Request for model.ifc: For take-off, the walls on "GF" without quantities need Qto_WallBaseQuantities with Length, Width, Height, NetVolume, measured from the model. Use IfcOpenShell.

First a look at what the model holds.

```python
import ifcopenshell
import ifcopenshell.util.element
import ifcopenshell.util.unit

model = ifcopenshell.open("model.ifc")
print(model.schema)
for unit_type in ("LENGTHUNIT", "AREAUNIT", "VOLUMEUNIT"):
    print(unit_type, ifcopenshell.util.unit.calculate_unit_scale(model, unit_type))
storey = next(s for s in model.by_type("IfcBuildingStorey") if s.Name == "GF")
walls = [e for e in ifcopenshell.util.element.get_decomposition(storey) if e.is_a("IfcWall")]
for e in sorted(walls, key=lambda e: e.id()):
    print(e.id(), e.is_a(), e.Name, list(ifcopenshell.util.element.get_psets(e, qtos_only=True)), sep=" | ")
```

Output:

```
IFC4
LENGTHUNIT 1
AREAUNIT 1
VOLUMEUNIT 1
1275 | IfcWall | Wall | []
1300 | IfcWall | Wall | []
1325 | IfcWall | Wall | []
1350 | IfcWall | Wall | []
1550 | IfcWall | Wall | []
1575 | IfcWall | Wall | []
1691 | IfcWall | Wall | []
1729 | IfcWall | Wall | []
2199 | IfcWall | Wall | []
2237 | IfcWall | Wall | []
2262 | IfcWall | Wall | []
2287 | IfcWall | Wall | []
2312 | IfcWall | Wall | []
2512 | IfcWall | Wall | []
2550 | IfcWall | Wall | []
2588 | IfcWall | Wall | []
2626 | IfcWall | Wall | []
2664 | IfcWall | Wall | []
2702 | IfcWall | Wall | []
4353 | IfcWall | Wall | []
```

```python
import ifcopenshell
import ifcopenshell.api.pset
import ifcopenshell.geom
import ifcopenshell.util.element
import ifcopenshell.util.shape
import ifcopenshell.util.unit

model = ifcopenshell.open("model.ifc")
unit_scale = ifcopenshell.util.unit.calculate_unit_scale(model)
volume_scale = ifcopenshell.util.unit.calculate_unit_scale(model, "VOLUMEUNIT")
settings = ifcopenshell.geom.settings()

storey = next(s for s in model.by_type("IfcBuildingStorey") if s.Name == "GF")
walls = [e for e in ifcopenshell.util.element.get_decomposition(storey) if e.is_a("IfcWall")]

for e in sorted(walls, key=lambda e: e.id()):
    if ifcopenshell.util.element.get_psets(e, qtos_only=True, should_inherit=False):
        continue
    # Geometry comes back in metres, in the element's own axes.
    shape = ifcopenshell.geom.create_shape(settings, e)
    values = {
        "Length": ifcopenshell.util.shape.get_x(shape.geometry) / unit_scale,
        "Width": ifcopenshell.util.shape.get_y(shape.geometry) / unit_scale,
        "Height": ifcopenshell.util.shape.get_z(shape.geometry) / unit_scale,
        "NetVolume": ifcopenshell.util.shape.get_volume(shape.geometry) / volume_scale,
    }
    qto = ifcopenshell.api.pset.add_qto(model, product=e, name="Qto_WallBaseQuantities")
    ifcopenshell.api.pset.edit_qto(model, qto=qto, properties=values)
    print(e.id(), {k: round(v, 3) for k, v in values.items()})

model.write("model_v2.ifc")
```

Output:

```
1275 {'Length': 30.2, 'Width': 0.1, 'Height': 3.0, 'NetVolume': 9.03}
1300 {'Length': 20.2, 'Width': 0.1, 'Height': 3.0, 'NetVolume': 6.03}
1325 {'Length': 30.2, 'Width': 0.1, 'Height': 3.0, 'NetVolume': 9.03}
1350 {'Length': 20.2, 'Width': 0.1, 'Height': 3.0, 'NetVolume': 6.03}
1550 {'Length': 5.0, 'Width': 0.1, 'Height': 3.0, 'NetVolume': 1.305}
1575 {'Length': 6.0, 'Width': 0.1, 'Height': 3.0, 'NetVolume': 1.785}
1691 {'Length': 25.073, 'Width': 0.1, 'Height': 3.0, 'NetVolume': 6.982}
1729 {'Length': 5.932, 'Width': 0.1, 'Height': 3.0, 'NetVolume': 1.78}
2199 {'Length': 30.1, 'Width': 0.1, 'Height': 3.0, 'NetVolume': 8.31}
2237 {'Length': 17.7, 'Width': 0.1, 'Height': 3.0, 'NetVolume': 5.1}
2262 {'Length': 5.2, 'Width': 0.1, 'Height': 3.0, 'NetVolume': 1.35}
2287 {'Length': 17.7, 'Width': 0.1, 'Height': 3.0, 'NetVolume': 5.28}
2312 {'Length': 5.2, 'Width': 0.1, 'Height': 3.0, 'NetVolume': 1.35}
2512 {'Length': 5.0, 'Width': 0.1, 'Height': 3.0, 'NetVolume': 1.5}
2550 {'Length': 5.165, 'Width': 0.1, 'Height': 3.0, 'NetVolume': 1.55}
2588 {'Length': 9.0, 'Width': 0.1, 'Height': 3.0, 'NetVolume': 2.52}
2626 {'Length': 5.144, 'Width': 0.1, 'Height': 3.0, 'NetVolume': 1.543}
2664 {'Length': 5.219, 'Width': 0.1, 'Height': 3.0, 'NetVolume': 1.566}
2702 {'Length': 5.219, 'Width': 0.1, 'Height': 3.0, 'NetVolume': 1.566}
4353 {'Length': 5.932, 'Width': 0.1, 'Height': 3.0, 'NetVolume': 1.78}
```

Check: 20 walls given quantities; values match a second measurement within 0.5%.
